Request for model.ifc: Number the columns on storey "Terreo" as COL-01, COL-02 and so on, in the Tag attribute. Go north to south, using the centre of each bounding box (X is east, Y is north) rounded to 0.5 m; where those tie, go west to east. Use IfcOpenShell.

First a look at what the model holds.

```python
import ifcopenshell
import ifcopenshell.util.element
import ifcopenshell.util.placement

model = ifcopenshell.open("model.ifc")
print(model.schema)
storey = next(s for s in model.by_type("IfcBuildingStorey") if s.Name == "Terreo")
columns = [e for e in ifcopenshell.util.element.get_decomposition(storey) if e.is_a("IfcColumn")]
for e in sorted(columns, key=lambda e: e.id()):
    origin = ifcopenshell.util.placement.get_local_placement(e.ObjectPlacement)[:3, 3]
    print(e.id(), e.Tag, e.Name, origin.round(2) + 0.0, sep=" | ")
```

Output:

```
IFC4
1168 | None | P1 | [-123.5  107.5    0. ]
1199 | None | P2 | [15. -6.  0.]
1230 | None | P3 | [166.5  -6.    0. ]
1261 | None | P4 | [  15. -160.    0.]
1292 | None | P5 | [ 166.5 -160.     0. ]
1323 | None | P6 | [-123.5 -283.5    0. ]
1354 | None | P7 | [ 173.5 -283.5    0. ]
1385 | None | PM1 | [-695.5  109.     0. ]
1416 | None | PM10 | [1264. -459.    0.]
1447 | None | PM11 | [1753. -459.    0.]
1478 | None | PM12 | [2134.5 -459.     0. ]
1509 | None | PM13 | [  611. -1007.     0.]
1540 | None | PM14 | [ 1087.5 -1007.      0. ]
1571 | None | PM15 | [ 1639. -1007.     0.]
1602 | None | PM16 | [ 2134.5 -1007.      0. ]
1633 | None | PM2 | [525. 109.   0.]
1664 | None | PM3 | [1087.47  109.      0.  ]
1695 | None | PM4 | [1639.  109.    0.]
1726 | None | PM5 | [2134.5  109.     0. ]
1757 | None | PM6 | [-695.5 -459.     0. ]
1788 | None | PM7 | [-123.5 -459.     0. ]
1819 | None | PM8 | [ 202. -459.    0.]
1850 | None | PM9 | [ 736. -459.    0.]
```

```python
import ifcopenshell
import ifcopenshell.geom
import ifcopenshell.util.element
import ifcopenshell.util.shape

model = ifcopenshell.open("model.ifc")
settings = ifcopenshell.geom.settings()
settings.set("use-world-coords", True)


def centre(element):
    shape = ifcopenshell.geom.create_shape(settings, element)
    return ifcopenshell.util.shape.get_bbox_centroid(shape.geometry)


storey = next(s for s in model.by_type("IfcBuildingStorey") if s.Name == "Terreo")
columns = [e for e in ifcopenshell.util.element.get_decomposition(storey) if e.is_a("IfcColumn")]

# Insertion points can sit at a corner or the storey origin, so sort by the geometry (in metres).
centres = {e: centre(e) for e in columns}
columns.sort(key=lambda e: (-round(centres[e][1] / 0.5), centres[e][0]))

for i, e in enumerate(columns, start=1):
    number = f"COL-{i:02d}"
    e.Tag = number
    print(e.id(), number)

model.write("model-out.ifc")
```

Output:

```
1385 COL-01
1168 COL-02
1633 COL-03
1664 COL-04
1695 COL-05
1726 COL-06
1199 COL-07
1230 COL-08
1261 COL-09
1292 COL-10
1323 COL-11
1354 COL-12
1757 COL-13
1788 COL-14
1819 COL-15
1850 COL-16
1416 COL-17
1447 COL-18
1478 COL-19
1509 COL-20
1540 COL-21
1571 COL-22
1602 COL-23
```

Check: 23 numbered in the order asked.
